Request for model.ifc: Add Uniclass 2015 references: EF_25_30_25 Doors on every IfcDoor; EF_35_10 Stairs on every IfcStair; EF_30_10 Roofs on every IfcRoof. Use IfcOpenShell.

First a look at what the model holds.

```python
import ifcopenshell

model = ifcopenshell.open("model.ifc")
print(model.schema)
print("classifications:", [c.Name for c in model.by_type("IfcClassification")])
for ifc_class in ("IfcDoor", "IfcRoof", "IfcStair", "IfcWall", "IfcWindow"):
    print(ifc_class, len(model.by_type(ifc_class)))
```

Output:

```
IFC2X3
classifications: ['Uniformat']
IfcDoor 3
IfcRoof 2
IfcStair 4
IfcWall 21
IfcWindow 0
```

```python
import ifcopenshell
import ifcopenshell.api.classification

model = ifcopenshell.open("model.ifc")

# IFC2X3 requires Source and Edition and has no link from the project to the system.
system = model.create_entity("IfcClassification", Source="NBS", Edition="2015", Name="Uniclass 2015")

codes = {
    "IfcDoor": ("EF_25_30_25", "Doors"),
    "IfcStair": ("EF_35_10", "Stairs"),
    "IfcRoof": ("EF_30_10", "Roofs"),
}
for ifc_class, (code, name) in codes.items():
    products = model.by_type(ifc_class)
    ifcopenshell.api.classification.add_reference(
        model, products=products, classification=system, identification=code, name=name
    )
    print(code, len(products))

model.write("model_edited.ifc")
```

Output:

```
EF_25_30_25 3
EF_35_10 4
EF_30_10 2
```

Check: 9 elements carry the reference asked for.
